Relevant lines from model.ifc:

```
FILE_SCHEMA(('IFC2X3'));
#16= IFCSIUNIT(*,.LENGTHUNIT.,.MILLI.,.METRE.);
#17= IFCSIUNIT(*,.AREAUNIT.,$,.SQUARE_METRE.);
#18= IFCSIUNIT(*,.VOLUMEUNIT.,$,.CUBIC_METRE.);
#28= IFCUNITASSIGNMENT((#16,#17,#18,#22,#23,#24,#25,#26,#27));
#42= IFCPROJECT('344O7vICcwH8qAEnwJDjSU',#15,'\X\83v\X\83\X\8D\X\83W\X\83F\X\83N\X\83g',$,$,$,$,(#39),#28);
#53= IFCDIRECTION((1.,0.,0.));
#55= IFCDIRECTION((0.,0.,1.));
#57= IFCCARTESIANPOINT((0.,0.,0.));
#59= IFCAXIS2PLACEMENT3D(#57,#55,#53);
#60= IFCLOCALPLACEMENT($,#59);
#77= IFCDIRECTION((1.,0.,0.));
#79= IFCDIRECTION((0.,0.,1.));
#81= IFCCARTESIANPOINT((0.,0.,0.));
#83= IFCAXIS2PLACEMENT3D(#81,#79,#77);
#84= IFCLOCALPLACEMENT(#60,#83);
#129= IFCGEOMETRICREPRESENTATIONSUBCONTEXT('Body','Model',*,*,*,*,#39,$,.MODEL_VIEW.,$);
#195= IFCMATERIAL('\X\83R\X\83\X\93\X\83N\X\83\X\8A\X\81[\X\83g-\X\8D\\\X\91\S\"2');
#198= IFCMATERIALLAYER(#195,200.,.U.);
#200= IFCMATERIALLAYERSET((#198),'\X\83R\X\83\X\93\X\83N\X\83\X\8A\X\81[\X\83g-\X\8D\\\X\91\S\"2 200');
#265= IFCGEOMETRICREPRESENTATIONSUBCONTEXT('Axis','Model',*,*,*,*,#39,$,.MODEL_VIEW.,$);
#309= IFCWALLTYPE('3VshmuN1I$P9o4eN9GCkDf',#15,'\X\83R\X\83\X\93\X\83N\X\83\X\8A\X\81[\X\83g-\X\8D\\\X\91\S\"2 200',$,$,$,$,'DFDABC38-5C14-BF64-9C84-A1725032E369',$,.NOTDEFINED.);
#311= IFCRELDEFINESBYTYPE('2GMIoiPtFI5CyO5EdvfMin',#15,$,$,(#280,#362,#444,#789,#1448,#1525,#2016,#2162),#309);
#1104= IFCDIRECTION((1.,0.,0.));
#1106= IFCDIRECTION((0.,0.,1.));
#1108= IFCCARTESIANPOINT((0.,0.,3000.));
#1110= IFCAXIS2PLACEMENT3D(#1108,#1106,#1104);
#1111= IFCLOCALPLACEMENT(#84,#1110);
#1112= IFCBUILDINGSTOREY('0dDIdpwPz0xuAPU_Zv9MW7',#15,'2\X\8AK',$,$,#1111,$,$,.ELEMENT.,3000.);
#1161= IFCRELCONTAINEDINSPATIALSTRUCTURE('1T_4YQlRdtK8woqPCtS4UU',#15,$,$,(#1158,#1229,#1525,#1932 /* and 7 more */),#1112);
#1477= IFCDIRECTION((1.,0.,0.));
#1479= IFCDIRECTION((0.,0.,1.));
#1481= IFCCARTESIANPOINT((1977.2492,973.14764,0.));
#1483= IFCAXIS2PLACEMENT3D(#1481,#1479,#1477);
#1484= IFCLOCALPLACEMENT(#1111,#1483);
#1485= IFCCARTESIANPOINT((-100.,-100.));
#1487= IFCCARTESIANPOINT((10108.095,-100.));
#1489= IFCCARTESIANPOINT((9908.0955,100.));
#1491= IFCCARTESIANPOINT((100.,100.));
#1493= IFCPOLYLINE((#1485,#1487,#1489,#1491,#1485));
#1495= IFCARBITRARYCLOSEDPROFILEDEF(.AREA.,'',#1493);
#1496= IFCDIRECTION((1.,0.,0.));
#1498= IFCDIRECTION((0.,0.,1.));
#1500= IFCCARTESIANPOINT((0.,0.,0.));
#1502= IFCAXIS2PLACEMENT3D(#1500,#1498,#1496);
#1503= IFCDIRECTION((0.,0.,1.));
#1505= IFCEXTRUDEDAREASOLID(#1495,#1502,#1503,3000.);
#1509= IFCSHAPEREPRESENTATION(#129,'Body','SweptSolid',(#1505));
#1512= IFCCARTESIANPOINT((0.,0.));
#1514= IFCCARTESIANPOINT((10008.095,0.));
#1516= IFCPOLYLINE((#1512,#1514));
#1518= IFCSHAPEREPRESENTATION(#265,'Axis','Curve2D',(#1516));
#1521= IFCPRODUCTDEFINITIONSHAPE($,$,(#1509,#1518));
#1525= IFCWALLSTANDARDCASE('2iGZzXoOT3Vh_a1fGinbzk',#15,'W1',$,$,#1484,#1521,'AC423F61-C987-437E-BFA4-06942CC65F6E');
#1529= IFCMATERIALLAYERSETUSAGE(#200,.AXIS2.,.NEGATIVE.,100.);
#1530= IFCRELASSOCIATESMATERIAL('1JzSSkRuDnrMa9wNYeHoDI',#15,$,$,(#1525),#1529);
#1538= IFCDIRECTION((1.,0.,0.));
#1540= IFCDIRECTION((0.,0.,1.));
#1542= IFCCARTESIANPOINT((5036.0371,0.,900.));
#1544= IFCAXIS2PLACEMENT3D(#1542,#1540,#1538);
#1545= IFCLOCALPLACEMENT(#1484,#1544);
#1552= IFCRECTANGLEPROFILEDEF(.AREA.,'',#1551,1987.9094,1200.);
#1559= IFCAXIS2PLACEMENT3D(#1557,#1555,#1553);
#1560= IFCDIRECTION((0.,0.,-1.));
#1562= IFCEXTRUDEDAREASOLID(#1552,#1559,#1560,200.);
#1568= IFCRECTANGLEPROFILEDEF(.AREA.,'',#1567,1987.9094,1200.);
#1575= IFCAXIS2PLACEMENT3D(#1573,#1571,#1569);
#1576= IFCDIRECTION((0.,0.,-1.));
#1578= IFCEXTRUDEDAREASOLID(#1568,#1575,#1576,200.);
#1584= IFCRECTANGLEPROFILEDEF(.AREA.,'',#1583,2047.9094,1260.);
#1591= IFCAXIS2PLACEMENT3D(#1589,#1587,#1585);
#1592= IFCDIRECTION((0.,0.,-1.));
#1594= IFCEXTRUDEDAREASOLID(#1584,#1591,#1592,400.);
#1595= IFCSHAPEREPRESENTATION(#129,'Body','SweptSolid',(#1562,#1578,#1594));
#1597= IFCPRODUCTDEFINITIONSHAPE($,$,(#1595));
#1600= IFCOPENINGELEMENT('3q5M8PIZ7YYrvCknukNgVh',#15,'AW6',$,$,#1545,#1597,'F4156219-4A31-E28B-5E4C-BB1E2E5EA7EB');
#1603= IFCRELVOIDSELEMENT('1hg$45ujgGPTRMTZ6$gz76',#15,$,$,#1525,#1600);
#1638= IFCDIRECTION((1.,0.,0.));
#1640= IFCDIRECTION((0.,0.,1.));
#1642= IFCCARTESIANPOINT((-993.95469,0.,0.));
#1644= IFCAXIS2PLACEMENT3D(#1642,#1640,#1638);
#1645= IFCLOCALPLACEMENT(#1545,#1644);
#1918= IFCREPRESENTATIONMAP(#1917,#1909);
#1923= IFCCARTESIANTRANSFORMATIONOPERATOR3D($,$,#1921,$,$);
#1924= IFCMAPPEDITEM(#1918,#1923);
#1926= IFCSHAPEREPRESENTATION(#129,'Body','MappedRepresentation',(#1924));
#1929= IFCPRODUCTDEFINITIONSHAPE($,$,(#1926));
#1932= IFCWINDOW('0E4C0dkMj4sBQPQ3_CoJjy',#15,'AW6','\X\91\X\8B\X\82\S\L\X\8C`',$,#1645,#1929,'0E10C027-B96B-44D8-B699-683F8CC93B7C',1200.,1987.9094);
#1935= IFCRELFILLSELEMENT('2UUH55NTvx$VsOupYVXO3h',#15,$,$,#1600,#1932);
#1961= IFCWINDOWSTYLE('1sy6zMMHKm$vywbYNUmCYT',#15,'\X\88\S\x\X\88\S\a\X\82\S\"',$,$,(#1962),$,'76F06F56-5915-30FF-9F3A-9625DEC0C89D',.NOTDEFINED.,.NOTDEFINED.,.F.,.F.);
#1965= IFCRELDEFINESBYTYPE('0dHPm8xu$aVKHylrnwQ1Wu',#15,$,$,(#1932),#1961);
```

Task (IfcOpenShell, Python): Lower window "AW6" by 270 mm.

```python
import numpy as np
import ifcopenshell
import ifcopenshell.api.geometry
import ifcopenshell.util.placement
import ifcopenshell.util.unit

model = ifcopenshell.open("model.ifc")
unit_scale = ifcopenshell.util.unit.calculate_unit_scale(model)

window = model.by_guid("0E4C0dkMj4sBQPQ3_CoJjy")
opening = window.FillsVoids[0].RelatingOpeningElement
dz = -270.0

shift = np.array([0.0, 0.0, dz])
# The window is placed relative to its opening, so it follows when the opening moves.
matrix = ifcopenshell.util.placement.get_local_placement(opening.ObjectPlacement)
matrix[:3, 3] += shift
ifcopenshell.api.geometry.edit_object_placement(
    model, product=opening, matrix=matrix, is_si=False, should_transform_children=True
)

print(f"moved by {dz * unit_scale:+.3f} m")

model.write("model_updated.ifc")
```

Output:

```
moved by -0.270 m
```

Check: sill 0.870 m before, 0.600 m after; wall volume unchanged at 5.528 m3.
